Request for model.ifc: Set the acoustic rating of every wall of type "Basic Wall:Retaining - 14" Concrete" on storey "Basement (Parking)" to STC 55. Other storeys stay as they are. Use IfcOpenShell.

First a look at what the model holds.

```python
import ifcopenshell
import ifcopenshell.util.element

model = ifcopenshell.open("model.ifc")
print(model.schema)
storey = next(s for s in model.by_type("IfcBuildingStorey") if s.Name == "Basement (Parking)")
walls = [e for e in ifcopenshell.util.element.get_decomposition(storey) if e.is_a("IfcWall")]
seen = {}
for e in walls:
    element_type = ifcopenshell.util.element.get_type(e)
    key = (element_type.Name if element_type != e and element_type else None, ifcopenshell.util.element.get_pset(e, "Pset_WallCommon", "AcousticRating"))
    seen[key] = seen.get(key, 0) + 1
for (name, value), count in sorted(seen.items(), key=str):
    print(count, "x", name, "|", value)
```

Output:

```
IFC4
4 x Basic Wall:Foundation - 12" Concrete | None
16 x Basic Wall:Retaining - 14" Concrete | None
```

```python
import ifcopenshell
import ifcopenshell.api.pset
import ifcopenshell.util.element

model = ifcopenshell.open("model.ifc")

storey = next(s for s in model.by_type("IfcBuildingStorey") if s.Name == "Basement (Parking)")
walls = [e for e in ifcopenshell.util.element.get_decomposition(storey) if e.is_a("IfcWall")]

count = 0
for e in walls:
    element_type = ifcopenshell.util.element.get_type(e)
    if element_type in (None, e) or element_type.Name != 'Basic Wall:Retaining - 14" Concrete':
        continue
    # add_pset returns the element's existing set when there is one.
    pset = ifcopenshell.api.pset.add_pset(model, product=e, name="Pset_WallCommon")
    ifcopenshell.api.pset.edit_pset(model, pset=pset, properties={"AcousticRating": "STC 55"})
    count += 1

print(count, "walls updated")

model.write("model_rev.ifc")
```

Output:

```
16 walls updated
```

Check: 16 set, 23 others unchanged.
